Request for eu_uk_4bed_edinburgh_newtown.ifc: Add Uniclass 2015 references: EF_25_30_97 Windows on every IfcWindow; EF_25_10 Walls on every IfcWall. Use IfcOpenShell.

First a look at what the model holds.

```python
import ifcopenshell

model = ifcopenshell.open("eu_uk_4bed_edinburgh_newtown.ifc")
print(model.schema)
print("classifications:", [c.Name for c in model.by_type("IfcClassification")])
for ifc_class in ("IfcDoor", "IfcRoof", "IfcStair", "IfcWall", "IfcWindow"):
    print(ifc_class, len(model.by_type(ifc_class)))
```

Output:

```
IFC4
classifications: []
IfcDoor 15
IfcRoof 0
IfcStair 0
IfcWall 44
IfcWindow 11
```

```python
import ifcopenshell
import ifcopenshell.api.classification

model = ifcopenshell.open("eu_uk_4bed_edinburgh_newtown.ifc")

system = ifcopenshell.api.classification.add_classification(model, classification="Uniclass 2015")

codes = {
    "IfcWindow": ("EF_25_30_97", "Windows"),
    "IfcWall": ("EF_25_10", "Walls"),
}
for ifc_class, (code, name) in codes.items():
    products = model.by_type(ifc_class)
    ifcopenshell.api.classification.add_reference(
        model, products=products, classification=system, identification=code, name=name
    )
    print(code, len(products))

model.write("eu_uk_4bed_edinburgh_newtown_updated.ifc")
```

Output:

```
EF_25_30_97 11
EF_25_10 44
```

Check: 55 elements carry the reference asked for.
